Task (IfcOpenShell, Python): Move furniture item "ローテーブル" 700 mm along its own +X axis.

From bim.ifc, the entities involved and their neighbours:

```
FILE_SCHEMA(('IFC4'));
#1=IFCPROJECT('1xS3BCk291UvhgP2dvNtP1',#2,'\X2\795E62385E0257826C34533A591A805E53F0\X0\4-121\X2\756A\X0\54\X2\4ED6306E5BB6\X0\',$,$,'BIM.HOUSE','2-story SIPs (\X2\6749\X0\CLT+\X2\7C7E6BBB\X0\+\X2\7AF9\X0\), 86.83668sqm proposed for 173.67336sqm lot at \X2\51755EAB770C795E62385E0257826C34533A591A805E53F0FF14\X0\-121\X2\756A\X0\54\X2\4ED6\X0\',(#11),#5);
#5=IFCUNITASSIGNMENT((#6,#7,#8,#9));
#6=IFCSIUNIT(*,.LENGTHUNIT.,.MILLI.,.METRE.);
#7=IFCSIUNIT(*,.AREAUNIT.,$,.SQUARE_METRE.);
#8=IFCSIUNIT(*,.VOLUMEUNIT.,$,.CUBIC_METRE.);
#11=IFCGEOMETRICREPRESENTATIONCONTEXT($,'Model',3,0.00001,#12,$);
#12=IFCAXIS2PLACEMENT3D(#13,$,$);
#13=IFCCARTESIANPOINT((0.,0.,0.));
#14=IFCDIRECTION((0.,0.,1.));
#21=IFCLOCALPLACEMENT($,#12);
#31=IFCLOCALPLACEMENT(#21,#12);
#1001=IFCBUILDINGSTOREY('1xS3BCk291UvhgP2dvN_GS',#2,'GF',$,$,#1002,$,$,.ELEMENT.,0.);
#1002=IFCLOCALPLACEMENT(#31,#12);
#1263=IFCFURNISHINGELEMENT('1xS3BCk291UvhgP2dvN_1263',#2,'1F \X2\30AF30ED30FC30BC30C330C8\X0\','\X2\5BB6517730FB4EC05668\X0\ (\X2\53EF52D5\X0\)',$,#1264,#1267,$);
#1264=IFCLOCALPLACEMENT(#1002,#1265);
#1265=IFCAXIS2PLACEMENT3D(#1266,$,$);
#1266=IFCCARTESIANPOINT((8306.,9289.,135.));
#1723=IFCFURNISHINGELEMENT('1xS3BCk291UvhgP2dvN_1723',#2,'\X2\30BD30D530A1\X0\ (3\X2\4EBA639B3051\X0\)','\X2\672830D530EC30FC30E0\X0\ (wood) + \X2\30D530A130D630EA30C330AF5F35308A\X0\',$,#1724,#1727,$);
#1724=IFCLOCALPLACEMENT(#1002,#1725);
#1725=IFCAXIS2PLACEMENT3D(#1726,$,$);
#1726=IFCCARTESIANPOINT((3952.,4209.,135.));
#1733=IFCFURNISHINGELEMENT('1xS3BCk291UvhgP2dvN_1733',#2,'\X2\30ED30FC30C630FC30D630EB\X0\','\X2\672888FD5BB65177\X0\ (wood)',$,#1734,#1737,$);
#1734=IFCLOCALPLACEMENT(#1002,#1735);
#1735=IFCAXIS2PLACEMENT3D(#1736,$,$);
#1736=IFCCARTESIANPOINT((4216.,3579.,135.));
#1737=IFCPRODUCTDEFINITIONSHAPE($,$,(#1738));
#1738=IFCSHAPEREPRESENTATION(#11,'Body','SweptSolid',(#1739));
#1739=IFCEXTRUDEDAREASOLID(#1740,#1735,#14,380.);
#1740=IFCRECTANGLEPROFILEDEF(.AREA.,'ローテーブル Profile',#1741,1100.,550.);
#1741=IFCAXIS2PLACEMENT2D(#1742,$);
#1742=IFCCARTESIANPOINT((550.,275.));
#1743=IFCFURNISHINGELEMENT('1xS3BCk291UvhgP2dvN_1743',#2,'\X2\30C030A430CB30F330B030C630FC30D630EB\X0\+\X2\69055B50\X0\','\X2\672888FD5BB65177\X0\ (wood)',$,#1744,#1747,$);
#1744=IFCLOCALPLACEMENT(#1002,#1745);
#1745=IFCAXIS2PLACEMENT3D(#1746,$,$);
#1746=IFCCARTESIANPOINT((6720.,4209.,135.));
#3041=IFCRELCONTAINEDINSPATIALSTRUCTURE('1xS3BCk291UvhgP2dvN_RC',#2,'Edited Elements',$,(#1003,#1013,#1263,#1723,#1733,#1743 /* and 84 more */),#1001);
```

```python
import ifcopenshell
import ifcopenshell.api.geometry
import ifcopenshell.util.placement
import ifcopenshell.util.unit

model = ifcopenshell.open("bim.ifc")
unit_scale = ifcopenshell.util.unit.calculate_unit_scale(model)

item = model.by_guid("1xS3BCk291UvhgP2dvN_1733")
matrix = ifcopenshell.util.placement.get_local_placement(item.ObjectPlacement)
matrix[:3, 3] += matrix[:3, 0] * 0.7 / unit_scale
ifcopenshell.api.geometry.edit_object_placement(model, product=item, matrix=matrix, is_si=False)

print(ifcopenshell.util.placement.get_local_placement(item.ObjectPlacement).round(3) + 0.0)

model.write("bim_updated.ifc")
```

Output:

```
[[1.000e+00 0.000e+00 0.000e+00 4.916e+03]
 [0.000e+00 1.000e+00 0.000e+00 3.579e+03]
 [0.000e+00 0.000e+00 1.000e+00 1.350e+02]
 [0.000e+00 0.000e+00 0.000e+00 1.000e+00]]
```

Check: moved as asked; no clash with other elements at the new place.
